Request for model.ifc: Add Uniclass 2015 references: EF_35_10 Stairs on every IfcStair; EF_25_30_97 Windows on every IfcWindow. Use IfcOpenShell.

First a look at what the model holds.

```python
import ifcopenshell

model = ifcopenshell.open("model.ifc")
print(model.schema)
print("classifications:", [c.Name for c in model.by_type("IfcClassification")])
for ifc_class in ("IfcDoor", "IfcRoof", "IfcStair", "IfcWall", "IfcWindow"):
    print(ifc_class, len(model.by_type(ifc_class)))
```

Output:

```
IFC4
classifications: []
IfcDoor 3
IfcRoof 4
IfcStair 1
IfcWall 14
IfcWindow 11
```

```python
import ifcopenshell
import ifcopenshell.api.classification

model = ifcopenshell.open("model.ifc")

system = ifcopenshell.api.classification.add_classification(model, classification="Uniclass 2015")

codes = {
    "IfcStair": ("EF_35_10", "Stairs"),
    "IfcWindow": ("EF_25_30_97", "Windows"),
}
for ifc_class, (code, name) in codes.items():
    products = model.by_type(ifc_class)
    ifcopenshell.api.classification.add_reference(
        model, products=products, classification=system, identification=code, name=name
    )
    print(code, len(products))

model.write("model_v2.ifc")
```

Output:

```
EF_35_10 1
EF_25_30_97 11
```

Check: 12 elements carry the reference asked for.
